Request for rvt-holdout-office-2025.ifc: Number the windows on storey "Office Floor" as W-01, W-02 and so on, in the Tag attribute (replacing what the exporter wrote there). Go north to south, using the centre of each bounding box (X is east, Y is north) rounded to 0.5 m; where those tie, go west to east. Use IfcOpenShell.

First a look at what the model holds.

```python
import ifcopenshell
import ifcopenshell.util.element
import ifcopenshell.util.placement

model = ifcopenshell.open("rvt-holdout-office-2025.ifc")
print(model.schema)
storey = next(s for s in model.by_type("IfcBuildingStorey") if s.Name == "Office Floor")
windows = [e for e in ifcopenshell.util.element.get_decomposition(storey) if e.is_a("IfcWindow")]
for e in sorted(windows, key=lambda e: e.id()):
    origin = ifcopenshell.util.placement.get_local_placement(e.ObjectPlacement)[:3, 3]
    print(e.id(), e.Tag, e.Name, origin.round(2) + 0.0, sep=" | ")
```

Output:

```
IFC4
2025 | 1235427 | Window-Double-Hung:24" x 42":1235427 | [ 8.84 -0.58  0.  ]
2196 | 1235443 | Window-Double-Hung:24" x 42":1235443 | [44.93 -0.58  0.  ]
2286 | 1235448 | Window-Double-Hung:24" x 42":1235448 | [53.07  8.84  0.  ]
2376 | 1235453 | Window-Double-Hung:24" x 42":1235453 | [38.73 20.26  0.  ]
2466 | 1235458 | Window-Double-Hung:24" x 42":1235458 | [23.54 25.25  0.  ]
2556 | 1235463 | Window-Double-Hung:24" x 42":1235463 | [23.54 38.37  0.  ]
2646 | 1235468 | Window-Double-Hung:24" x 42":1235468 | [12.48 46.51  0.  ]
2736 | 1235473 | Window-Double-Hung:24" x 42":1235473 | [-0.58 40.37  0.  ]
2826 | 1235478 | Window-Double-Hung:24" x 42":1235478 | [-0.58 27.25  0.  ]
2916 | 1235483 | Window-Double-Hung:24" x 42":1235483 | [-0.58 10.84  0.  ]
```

```python
import ifcopenshell
import ifcopenshell.geom
import ifcopenshell.util.element
import ifcopenshell.util.shape

model = ifcopenshell.open("rvt-holdout-office-2025.ifc")
settings = ifcopenshell.geom.settings()
settings.set("use-world-coords", True)


def centre(element):
    shape = ifcopenshell.geom.create_shape(settings, element)
    return ifcopenshell.util.shape.get_bbox_centroid(shape.geometry)


storey = next(s for s in model.by_type("IfcBuildingStorey") if s.Name == "Office Floor")
windows = [e for e in ifcopenshell.util.element.get_decomposition(storey) if e.is_a("IfcWindow")]

# Insertion points can sit at a corner or the storey origin, so sort by the geometry (in metres).
centres = {e: centre(e) for e in windows}
windows.sort(key=lambda e: (-round(centres[e][1] / 0.5), centres[e][0]))

for i, e in enumerate(windows, start=1):
    number = f"W-{i:02d}"
    e.Tag = number
    print(e.id(), number)

model.write("rvt-holdout-office-2025_updated.ifc")
```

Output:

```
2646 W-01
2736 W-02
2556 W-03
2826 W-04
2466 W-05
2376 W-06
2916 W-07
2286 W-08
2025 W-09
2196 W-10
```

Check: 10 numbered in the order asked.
